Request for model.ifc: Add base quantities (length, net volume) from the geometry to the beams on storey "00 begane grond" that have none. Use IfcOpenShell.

First a look at what the model holds.

```python
import ifcopenshell
import ifcopenshell.util.element
import ifcopenshell.util.unit

model = ifcopenshell.open("model.ifc")
print(model.schema)
for unit_type in ("LENGTHUNIT", "AREAUNIT", "VOLUMEUNIT"):
    print(unit_type, ifcopenshell.util.unit.calculate_unit_scale(model, unit_type))
storey = next(s for s in model.by_type("IfcBuildingStorey") if s.Name == "00 begane grond")
beams = [e for e in ifcopenshell.util.element.get_decomposition(storey) if e.is_a("IfcBeam")]
for e in sorted(beams, key=lambda e: e.id()):
    print(e.id(), e.is_a(), e.Name, list(ifcopenshell.util.element.get_psets(e, qtos_only=True)), sep=" | ")
```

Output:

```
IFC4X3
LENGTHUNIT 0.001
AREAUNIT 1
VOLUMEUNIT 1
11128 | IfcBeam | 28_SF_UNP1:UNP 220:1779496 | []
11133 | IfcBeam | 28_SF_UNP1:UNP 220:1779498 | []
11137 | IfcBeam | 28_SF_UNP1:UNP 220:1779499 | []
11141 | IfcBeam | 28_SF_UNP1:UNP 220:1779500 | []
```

```python
import ifcopenshell
import ifcopenshell.api.pset
import ifcopenshell.geom
import ifcopenshell.util.element
import ifcopenshell.util.shape
import ifcopenshell.util.unit

model = ifcopenshell.open("model.ifc")
unit_scale = ifcopenshell.util.unit.calculate_unit_scale(model)
volume_scale = ifcopenshell.util.unit.calculate_unit_scale(model, "VOLUMEUNIT")
settings = ifcopenshell.geom.settings()

storey = next(s for s in model.by_type("IfcBuildingStorey") if s.Name == "00 begane grond")
beams = [e for e in ifcopenshell.util.element.get_decomposition(storey) if e.is_a("IfcBeam")]

for e in sorted(beams, key=lambda e: e.id()):
    if ifcopenshell.util.element.get_psets(e, qtos_only=True, should_inherit=False):
        continue
    # Geometry comes back in metres, in the element's own axes.
    shape = ifcopenshell.geom.create_shape(settings, e)
    values = {
        "Length": ifcopenshell.util.shape.get_max_xyz(shape.geometry) / unit_scale,
        "NetVolume": ifcopenshell.util.shape.get_volume(shape.geometry) / volume_scale,
    }
    qto = ifcopenshell.api.pset.add_qto(model, product=e, name="Qto_BeamBaseQuantities")
    ifcopenshell.api.pset.edit_qto(model, qto=qto, properties=values)
    print(e.id(), {k: round(v, 3) for k, v in values.items()})

model.write("model_v2.ifc")
```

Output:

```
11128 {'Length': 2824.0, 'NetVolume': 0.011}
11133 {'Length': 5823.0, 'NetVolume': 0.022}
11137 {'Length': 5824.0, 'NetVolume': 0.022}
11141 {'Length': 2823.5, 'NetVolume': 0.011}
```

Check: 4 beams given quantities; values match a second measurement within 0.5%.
